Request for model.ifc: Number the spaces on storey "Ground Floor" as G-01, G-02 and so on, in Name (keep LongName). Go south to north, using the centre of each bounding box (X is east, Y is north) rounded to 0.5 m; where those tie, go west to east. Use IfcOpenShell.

First a look at what the model holds.

```python
import ifcopenshell
import ifcopenshell.util.element
import ifcopenshell.util.placement

model = ifcopenshell.open("model.ifc")
print(model.schema)
storey = next(s for s in model.by_type("IfcBuildingStorey") if s.Name == "Ground Floor")
spaces = [e for e in ifcopenshell.util.element.get_decomposition(storey) if e.is_a("IfcSpace")]
for e in sorted(spaces, key=lambda e: e.id()):
    origin = ifcopenshell.util.placement.get_local_placement(e.ObjectPlacement)[:3, 3]
    print(e.id(), e.Name, e.LongName, origin.round(2) + 0.0, sep=" | ")
```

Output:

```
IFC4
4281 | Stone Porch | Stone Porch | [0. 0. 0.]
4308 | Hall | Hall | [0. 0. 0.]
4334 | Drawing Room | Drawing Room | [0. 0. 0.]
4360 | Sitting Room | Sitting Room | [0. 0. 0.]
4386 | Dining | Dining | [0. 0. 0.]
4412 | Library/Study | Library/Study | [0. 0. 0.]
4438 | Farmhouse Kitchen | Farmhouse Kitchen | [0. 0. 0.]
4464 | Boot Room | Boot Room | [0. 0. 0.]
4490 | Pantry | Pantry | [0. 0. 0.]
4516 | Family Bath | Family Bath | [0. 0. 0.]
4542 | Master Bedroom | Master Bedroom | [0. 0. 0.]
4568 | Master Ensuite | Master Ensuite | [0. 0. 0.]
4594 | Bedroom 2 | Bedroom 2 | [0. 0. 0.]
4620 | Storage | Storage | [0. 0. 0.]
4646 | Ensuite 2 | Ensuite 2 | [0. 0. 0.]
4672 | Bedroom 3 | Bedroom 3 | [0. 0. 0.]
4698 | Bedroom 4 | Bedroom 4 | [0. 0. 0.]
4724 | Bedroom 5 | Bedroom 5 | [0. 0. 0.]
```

```python
import ifcopenshell
import ifcopenshell.geom
import ifcopenshell.util.element
import ifcopenshell.util.shape

model = ifcopenshell.open("model.ifc")
settings = ifcopenshell.geom.settings()
settings.set("use-world-coords", True)


def centre(element):
    shape = ifcopenshell.geom.create_shape(settings, element)
    return ifcopenshell.util.shape.get_bbox_centroid(shape.geometry)


storey = next(s for s in model.by_type("IfcBuildingStorey") if s.Name == "Ground Floor")
spaces = [e for e in ifcopenshell.util.element.get_decomposition(storey) if e.is_a("IfcSpace")]

# Insertion points can sit at a corner or the storey origin, so sort by the geometry (in metres).
centres = {e: centre(e) for e in spaces}
spaces.sort(key=lambda e: (round(centres[e][1] / 0.5), centres[e][0]))

for i, e in enumerate(spaces, start=1):
    number = f"G-{i:02d}"
    e.Name = number
    print(e.id(), number)

model.write("model_edited.ifc")
```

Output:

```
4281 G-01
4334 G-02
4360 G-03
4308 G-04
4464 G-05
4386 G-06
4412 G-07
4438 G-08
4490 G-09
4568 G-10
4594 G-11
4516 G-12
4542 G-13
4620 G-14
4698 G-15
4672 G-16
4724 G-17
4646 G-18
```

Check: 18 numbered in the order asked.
